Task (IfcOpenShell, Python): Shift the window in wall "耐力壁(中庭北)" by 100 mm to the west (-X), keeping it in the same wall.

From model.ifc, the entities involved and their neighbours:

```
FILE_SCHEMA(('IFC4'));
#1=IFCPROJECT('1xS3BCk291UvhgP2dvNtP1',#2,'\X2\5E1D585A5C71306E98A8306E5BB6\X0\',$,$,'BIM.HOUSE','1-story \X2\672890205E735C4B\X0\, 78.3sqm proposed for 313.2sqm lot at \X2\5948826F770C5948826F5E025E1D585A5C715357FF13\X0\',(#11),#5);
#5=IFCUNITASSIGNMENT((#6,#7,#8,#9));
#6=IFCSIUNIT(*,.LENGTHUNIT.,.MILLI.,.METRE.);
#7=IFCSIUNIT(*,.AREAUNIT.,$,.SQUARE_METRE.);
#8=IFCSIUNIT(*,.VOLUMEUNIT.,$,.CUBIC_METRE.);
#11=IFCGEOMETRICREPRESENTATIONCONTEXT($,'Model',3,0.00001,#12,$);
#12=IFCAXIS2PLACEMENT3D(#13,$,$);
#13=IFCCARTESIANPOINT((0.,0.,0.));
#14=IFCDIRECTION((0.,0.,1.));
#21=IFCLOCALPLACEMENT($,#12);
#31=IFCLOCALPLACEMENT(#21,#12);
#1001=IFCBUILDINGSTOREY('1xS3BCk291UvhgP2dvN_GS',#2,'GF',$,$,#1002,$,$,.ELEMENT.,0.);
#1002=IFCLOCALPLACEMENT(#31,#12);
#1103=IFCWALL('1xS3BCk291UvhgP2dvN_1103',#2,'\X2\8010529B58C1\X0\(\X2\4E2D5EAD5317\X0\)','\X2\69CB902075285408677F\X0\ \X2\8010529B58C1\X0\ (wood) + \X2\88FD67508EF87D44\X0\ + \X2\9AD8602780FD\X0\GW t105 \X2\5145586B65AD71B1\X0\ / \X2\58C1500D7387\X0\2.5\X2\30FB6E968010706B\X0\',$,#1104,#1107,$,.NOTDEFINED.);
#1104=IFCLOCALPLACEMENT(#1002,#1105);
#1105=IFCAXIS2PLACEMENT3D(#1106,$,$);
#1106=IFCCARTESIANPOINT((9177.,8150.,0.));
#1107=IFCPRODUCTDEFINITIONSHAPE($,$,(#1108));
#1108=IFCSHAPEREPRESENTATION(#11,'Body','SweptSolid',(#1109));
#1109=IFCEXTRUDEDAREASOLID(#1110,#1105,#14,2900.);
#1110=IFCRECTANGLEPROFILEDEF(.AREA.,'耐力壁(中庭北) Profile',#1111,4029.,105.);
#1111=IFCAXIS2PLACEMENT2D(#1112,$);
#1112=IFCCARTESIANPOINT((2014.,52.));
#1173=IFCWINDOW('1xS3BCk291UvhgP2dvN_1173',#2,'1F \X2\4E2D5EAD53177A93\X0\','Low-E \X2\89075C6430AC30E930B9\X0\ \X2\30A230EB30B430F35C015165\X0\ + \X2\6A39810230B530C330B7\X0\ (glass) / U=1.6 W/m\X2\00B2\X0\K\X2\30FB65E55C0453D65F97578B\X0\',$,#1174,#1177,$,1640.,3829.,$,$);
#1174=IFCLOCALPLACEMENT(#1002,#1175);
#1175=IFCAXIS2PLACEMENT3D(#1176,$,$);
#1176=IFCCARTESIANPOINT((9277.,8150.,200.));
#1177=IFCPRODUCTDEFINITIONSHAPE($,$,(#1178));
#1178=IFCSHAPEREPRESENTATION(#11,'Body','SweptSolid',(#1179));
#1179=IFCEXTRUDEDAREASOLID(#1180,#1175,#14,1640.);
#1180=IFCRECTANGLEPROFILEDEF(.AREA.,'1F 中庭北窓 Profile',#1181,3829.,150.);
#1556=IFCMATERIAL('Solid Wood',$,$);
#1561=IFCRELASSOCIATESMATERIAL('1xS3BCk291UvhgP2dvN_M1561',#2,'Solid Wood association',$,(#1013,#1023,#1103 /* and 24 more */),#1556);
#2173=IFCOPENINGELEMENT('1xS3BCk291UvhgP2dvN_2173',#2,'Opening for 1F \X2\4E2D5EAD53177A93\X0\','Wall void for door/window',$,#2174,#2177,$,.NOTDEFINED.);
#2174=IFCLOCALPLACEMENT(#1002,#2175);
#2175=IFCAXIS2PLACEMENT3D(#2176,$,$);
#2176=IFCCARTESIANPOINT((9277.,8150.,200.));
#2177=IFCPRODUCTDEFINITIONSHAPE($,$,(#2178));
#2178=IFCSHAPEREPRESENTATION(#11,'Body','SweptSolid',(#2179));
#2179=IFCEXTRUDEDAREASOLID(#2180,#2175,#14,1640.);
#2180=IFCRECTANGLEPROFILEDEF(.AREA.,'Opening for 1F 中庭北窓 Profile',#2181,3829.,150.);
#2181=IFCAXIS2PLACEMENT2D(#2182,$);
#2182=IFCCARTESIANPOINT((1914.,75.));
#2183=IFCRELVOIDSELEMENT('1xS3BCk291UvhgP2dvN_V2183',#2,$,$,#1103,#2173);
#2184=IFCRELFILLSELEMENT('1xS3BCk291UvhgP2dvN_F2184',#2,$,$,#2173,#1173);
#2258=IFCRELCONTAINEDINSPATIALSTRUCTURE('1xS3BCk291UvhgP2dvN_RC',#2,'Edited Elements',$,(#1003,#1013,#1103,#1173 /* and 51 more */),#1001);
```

```python
import ifcopenshell
import ifcopenshell.api.geometry
import ifcopenshell.util.placement
import ifcopenshell.util.unit

model = ifcopenshell.open("model.ifc")
unit_scale = ifcopenshell.util.unit.calculate_unit_scale(model)

window = model.by_guid("1xS3BCk291UvhgP2dvN_1173")
opening = window.FillsVoids[0].RelatingOpeningElement
wall = opening.VoidsElements[0].RelatingBuildingElement

wall_matrix = ifcopenshell.util.placement.get_local_placement(wall.ObjectPlacement)
shift = wall_matrix[:3, 0] * -0.1 / unit_scale
before = ifcopenshell.util.placement.get_local_placement(window.ObjectPlacement)[:3, 3].copy()

# The window is not placed relative to its opening, so move both.
for product in (opening, window):
    matrix = ifcopenshell.util.placement.get_local_placement(product.ObjectPlacement)
    matrix[:3, 3] += shift
    ifcopenshell.api.geometry.edit_object_placement(model, product=product, matrix=matrix, is_si=False)

after = ifcopenshell.util.placement.get_local_placement(window.ObjectPlacement)[:3, 3]
print("window moved by", (after - before).round(3) + 0.0)

model.write("model_rev.ifc")
```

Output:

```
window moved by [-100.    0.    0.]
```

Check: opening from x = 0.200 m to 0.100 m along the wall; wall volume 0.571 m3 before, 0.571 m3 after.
